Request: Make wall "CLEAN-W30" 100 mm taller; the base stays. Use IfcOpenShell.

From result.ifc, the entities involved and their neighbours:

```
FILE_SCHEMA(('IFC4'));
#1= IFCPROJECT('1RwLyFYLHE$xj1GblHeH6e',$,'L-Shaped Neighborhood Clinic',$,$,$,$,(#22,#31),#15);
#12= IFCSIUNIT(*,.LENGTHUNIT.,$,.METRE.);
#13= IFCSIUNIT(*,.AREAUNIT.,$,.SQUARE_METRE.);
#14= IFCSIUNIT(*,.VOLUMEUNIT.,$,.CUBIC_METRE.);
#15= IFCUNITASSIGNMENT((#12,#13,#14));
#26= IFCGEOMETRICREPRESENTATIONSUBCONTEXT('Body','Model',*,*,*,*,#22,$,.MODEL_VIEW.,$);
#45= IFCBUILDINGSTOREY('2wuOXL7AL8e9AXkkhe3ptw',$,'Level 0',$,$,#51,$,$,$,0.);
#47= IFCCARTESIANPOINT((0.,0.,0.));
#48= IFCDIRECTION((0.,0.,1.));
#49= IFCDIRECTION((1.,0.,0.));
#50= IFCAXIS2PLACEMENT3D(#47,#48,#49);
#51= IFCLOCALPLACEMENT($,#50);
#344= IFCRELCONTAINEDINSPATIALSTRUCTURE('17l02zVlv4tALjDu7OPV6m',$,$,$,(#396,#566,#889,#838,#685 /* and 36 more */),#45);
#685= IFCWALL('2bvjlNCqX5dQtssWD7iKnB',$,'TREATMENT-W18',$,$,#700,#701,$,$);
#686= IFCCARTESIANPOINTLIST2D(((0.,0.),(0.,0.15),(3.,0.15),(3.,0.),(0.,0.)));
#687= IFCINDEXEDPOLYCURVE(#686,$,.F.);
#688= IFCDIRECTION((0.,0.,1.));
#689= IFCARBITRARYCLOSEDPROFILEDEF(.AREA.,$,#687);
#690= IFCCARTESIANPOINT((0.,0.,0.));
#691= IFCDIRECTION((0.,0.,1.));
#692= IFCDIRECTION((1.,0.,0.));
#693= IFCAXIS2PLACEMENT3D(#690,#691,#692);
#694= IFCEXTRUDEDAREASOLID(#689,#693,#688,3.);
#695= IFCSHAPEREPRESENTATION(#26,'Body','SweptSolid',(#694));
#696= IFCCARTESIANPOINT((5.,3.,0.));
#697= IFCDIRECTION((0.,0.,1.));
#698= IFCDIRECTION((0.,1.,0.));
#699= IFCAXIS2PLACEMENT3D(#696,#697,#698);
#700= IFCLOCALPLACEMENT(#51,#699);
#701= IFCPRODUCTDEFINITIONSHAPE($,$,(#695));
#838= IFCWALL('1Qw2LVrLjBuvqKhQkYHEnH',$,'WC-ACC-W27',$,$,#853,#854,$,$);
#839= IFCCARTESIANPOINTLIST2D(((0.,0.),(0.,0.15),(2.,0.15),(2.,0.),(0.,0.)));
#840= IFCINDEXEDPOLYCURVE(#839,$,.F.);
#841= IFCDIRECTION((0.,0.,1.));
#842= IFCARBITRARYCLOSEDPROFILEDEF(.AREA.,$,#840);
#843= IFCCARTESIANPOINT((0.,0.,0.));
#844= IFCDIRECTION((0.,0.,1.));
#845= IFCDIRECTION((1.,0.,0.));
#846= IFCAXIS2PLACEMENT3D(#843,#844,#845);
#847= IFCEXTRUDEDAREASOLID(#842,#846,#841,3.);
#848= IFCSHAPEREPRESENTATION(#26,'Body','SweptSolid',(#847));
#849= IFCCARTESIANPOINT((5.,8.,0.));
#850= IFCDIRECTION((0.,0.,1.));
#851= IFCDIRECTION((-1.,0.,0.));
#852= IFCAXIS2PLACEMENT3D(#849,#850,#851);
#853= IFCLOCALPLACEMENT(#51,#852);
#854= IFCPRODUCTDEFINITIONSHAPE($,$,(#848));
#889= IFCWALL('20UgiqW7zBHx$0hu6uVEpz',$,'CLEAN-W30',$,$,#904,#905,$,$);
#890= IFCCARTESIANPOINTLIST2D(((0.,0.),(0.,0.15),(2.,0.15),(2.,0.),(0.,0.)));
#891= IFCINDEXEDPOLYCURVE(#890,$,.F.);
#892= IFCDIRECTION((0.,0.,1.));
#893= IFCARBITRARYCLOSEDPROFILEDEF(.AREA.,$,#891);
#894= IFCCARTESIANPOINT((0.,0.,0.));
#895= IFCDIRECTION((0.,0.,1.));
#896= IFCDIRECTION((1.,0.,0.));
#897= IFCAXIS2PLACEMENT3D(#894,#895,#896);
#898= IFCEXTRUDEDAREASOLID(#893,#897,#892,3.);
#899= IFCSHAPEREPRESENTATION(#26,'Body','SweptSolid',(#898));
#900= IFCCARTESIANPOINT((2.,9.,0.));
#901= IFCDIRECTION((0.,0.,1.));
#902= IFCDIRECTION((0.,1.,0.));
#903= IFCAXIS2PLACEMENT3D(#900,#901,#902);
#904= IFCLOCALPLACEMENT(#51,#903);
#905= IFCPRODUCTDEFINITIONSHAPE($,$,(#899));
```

```python
import ifcopenshell
import ifcopenshell.geom
import ifcopenshell.util.representation
import ifcopenshell.util.shape
import ifcopenshell.util.unit

model = ifcopenshell.open("result.ifc")
unit_scale = ifcopenshell.util.unit.calculate_unit_scale(model)
settings = ifcopenshell.geom.settings()


def volume(element):
    """Net volume in cubic metres, openings subtracted."""
    shape = ifcopenshell.geom.create_shape(settings, element)
    return ifcopenshell.util.shape.get_volume(shape.geometry)


wall = model.by_guid("20UgiqW7zBHx$0hu6uVEpz")
before = volume(wall)

body = ifcopenshell.util.representation.get_representation(wall, "Model", "Body")
solid = body.Items[0]
old_height = solid.Depth
solid.Depth += 0.1 / unit_scale
after = volume(wall)

print(f"height {old_height:g} -> {solid.Depth:g}, volume {before:.3f} -> {after:.3f} m3")

model.write("result_updated.ifc")
```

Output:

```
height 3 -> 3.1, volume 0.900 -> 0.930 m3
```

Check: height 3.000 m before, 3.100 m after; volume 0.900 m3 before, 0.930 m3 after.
